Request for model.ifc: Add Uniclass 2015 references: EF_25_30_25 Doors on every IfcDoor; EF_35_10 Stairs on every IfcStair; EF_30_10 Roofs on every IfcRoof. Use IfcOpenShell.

First a look at what the model holds.

```python
import ifcopenshell

model = ifcopenshell.open("model.ifc")
print(model.schema)
print("classifications:", [c.Name for c in model.by_type("IfcClassification")])
for ifc_class in ("IfcDoor", "IfcRoof", "IfcStair", "IfcWall", "IfcWindow"):
    print(ifc_class, len(model.by_type(ifc_class)))
```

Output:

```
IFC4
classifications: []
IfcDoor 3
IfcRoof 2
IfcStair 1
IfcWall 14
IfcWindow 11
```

```python
import ifcopenshell
import ifcopenshell.api.classification

model = ifcopenshell.open("model.ifc")

system = ifcopenshell.api.classification.add_classification(model, classification="Uniclass 2015")

codes = {
    "IfcDoor": ("EF_25_30_25", "Doors"),
    "IfcStair": ("EF_35_10", "Stairs"),
    "IfcRoof": ("EF_30_10", "Roofs"),
}
for ifc_class, (code, name) in codes.items():
    products = model.by_type(ifc_class)
    ifcopenshell.api.classification.add_reference(
        model, products=products, classification=system, identification=code, name=name
    )
    print(code, len(products))

model.write("model-out.ifc")
```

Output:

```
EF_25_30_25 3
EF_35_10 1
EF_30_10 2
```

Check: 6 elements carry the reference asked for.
